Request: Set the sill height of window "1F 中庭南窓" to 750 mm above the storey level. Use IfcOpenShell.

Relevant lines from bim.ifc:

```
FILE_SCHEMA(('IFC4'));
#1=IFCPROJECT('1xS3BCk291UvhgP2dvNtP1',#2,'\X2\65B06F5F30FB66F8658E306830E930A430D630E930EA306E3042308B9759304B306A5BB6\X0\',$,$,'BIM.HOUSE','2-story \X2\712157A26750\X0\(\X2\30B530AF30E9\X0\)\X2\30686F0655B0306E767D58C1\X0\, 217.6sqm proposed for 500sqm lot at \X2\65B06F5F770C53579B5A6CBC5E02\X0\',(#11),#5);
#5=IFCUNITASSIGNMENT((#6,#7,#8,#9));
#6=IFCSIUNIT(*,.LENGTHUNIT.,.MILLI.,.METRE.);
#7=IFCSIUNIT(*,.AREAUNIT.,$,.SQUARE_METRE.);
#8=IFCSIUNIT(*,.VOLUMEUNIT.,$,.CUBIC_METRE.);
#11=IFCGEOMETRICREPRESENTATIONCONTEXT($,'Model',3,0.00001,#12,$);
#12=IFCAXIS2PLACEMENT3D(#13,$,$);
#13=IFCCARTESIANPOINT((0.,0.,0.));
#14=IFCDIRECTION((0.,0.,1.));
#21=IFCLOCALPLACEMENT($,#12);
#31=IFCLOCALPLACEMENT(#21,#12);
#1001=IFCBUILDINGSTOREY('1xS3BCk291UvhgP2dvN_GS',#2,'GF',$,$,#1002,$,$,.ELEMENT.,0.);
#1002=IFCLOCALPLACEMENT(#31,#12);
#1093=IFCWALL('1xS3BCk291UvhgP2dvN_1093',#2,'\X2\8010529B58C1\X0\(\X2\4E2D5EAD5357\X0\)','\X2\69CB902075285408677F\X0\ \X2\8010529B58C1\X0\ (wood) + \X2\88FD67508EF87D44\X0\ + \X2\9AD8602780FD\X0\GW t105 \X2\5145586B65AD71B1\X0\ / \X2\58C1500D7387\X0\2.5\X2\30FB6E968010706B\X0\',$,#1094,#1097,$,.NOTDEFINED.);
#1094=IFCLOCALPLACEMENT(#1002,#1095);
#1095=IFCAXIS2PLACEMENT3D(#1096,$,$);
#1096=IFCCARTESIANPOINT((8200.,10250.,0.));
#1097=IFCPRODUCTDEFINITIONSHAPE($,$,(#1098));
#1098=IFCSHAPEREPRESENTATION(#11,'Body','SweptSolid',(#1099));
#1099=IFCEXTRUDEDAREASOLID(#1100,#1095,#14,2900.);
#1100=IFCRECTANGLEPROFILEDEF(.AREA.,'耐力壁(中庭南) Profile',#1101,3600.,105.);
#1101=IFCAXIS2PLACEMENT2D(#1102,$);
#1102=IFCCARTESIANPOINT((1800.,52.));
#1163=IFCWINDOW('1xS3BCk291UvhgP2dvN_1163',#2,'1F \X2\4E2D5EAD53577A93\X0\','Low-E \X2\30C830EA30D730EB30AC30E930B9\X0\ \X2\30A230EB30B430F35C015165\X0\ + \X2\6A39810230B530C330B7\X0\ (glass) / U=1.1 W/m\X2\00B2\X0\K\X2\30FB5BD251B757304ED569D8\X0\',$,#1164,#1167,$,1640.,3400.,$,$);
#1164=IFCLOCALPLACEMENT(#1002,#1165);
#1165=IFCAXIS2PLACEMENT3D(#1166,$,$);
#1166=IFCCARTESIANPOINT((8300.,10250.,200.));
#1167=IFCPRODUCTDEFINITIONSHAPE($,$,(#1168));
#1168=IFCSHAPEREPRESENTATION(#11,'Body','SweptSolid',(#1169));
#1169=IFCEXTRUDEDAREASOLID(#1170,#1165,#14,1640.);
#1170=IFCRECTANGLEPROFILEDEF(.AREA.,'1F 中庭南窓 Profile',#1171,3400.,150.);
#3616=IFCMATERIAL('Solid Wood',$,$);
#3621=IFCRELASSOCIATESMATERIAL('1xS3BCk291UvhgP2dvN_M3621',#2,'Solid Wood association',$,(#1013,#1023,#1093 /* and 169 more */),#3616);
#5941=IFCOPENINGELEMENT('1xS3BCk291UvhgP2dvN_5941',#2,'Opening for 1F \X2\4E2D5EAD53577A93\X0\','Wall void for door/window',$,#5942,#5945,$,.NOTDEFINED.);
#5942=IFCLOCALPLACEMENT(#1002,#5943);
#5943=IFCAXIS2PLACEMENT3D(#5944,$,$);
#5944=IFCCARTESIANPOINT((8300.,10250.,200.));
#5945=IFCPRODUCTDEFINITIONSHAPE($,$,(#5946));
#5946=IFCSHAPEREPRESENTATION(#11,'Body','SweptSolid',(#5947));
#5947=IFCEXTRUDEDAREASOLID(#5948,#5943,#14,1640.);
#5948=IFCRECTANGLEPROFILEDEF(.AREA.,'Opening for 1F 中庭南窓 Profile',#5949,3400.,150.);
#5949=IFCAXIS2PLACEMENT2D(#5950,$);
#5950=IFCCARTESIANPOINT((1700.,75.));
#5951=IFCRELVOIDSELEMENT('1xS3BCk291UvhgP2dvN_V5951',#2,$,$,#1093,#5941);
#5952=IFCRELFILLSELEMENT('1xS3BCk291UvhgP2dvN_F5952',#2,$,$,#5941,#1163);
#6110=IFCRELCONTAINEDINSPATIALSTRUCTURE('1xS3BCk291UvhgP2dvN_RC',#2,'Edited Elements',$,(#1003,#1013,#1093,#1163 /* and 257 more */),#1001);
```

```python
import numpy as np
import ifcopenshell
import ifcopenshell.api.geometry
import ifcopenshell.geom
import ifcopenshell.util.element
import ifcopenshell.util.placement
import ifcopenshell.util.shape
import ifcopenshell.util.unit

model = ifcopenshell.open("bim.ifc")
unit_scale = ifcopenshell.util.unit.calculate_unit_scale(model)

window = model.by_guid("1xS3BCk291UvhgP2dvN_1163")
opening = window.FillsVoids[0].RelatingOpeningElement
storey = ifcopenshell.util.element.get_container(window, ifc_class="IfcBuildingStorey")
level = ifcopenshell.util.placement.get_local_placement(storey.ObjectPlacement)[2, 3]

# The opening's origin need not be at the sill, so measure its lowest point.
shape = ifcopenshell.geom.create_shape(ifcopenshell.geom.settings(), opening)
bottom = ifcopenshell.util.shape.get_shape_bottom_elevation(shape, shape.geometry) / unit_scale
dz = level + 0.75 / unit_scale - bottom

shift = np.array([0.0, 0.0, dz])
# The window is not placed relative to its opening, so move both.
for product in (opening, window):
    matrix = ifcopenshell.util.placement.get_local_placement(product.ObjectPlacement)
    matrix[:3, 3] += shift
    ifcopenshell.api.geometry.edit_object_placement(model, product=product, matrix=matrix, is_si=False)

print(f"moved by {dz * unit_scale:+.3f} m")

model.write("bim_updated.ifc")
```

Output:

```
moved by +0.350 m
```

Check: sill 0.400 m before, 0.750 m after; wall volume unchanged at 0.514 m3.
